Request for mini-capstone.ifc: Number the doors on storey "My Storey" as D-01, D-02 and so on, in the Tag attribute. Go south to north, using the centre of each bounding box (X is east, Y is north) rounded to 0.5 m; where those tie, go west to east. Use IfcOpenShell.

First a look at what the model holds.

```python
import ifcopenshell
import ifcopenshell.util.element
import ifcopenshell.util.placement

model = ifcopenshell.open("mini-capstone.ifc")
print(model.schema)
storey = next(s for s in model.by_type("IfcBuildingStorey") if s.Name == "My Storey")
doors = [e for e in ifcopenshell.util.element.get_decomposition(storey) if e.is_a("IfcDoor")]
for e in sorted(doors, key=lambda e: e.id()):
    origin = ifcopenshell.util.placement.get_local_placement(e.ObjectPlacement)[:3, 3]
    print(e.id(), e.Tag, e.Name, origin.round(2) + 0.0, sep=" | ")
```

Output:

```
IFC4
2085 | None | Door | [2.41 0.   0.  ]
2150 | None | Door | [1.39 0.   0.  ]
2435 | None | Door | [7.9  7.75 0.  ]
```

```python
import ifcopenshell
import ifcopenshell.geom
import ifcopenshell.util.element
import ifcopenshell.util.shape

model = ifcopenshell.open("mini-capstone.ifc")
settings = ifcopenshell.geom.settings()
settings.set("use-world-coords", True)


def centre(element):
    shape = ifcopenshell.geom.create_shape(settings, element)
    return ifcopenshell.util.shape.get_bbox_centroid(shape.geometry)


storey = next(s for s in model.by_type("IfcBuildingStorey") if s.Name == "My Storey")
doors = [e for e in ifcopenshell.util.element.get_decomposition(storey) if e.is_a("IfcDoor")]

# Insertion points can sit at a corner or the storey origin, so sort by the geometry (in metres).
centres = {e: centre(e) for e in doors}
doors.sort(key=lambda e: (round(centres[e][1] / 0.5), centres[e][0]))

for i, e in enumerate(doors, start=1):
    number = f"D-{i:02d}"
    e.Tag = number
    print(e.id(), number)

model.write("mini-capstone_v2.ifc")
```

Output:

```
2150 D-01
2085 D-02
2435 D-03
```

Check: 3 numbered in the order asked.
